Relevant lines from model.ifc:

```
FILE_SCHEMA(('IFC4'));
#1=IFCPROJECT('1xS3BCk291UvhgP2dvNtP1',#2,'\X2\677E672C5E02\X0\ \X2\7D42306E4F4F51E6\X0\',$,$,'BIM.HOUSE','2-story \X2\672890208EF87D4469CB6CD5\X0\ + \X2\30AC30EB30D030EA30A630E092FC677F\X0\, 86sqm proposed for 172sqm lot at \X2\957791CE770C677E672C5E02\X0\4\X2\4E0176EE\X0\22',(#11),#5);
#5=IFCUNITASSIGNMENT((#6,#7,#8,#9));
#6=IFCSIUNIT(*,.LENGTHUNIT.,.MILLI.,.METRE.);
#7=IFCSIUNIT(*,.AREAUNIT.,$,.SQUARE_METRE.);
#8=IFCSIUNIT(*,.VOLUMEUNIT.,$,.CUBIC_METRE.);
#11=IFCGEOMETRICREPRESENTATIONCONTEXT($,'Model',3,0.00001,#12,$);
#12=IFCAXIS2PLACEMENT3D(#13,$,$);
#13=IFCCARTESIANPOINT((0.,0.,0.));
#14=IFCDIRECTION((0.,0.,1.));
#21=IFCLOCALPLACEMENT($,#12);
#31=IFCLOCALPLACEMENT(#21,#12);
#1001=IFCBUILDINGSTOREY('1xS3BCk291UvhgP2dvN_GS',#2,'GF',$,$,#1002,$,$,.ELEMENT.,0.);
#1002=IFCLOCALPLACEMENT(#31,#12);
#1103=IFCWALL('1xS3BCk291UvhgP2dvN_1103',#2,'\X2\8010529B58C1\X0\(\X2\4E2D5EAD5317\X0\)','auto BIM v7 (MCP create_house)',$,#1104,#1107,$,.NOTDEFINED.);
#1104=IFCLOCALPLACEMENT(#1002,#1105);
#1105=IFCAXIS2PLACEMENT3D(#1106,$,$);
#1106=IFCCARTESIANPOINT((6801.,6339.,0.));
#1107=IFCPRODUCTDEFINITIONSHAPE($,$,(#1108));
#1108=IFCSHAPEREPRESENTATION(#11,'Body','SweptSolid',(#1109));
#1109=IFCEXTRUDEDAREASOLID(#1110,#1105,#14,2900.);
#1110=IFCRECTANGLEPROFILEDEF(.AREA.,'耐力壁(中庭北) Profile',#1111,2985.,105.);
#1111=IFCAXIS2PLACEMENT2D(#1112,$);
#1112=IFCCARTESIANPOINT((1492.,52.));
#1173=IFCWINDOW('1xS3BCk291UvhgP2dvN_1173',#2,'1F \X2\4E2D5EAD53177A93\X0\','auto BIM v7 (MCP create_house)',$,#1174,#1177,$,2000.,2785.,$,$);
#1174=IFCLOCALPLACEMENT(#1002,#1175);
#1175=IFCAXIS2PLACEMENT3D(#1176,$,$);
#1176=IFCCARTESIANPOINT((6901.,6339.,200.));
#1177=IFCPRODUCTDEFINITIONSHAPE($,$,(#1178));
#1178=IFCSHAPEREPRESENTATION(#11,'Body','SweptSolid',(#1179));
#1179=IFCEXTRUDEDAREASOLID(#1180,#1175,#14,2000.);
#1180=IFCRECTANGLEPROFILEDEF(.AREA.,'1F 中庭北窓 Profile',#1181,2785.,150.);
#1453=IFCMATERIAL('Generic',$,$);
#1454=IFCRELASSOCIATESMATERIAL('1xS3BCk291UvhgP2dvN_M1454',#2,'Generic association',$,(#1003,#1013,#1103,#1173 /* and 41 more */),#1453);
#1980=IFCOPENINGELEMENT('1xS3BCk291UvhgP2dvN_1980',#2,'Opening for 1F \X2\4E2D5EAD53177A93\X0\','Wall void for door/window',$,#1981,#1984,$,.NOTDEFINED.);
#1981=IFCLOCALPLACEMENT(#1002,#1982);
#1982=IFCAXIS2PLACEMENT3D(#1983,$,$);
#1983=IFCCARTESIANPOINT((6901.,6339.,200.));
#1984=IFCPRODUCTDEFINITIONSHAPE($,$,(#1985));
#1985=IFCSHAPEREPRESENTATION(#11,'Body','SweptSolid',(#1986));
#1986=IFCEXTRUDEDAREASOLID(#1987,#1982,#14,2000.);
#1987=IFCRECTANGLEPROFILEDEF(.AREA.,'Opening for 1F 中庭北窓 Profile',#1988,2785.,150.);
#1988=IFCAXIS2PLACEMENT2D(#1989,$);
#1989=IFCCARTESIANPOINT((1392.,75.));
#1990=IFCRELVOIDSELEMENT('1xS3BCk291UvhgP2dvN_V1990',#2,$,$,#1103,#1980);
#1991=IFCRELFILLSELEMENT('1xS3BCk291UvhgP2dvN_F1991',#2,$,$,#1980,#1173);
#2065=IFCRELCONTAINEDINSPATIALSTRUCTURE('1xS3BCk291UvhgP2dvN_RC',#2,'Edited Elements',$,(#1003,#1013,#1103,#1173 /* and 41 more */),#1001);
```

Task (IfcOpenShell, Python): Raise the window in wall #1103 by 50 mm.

```python
import numpy as np
import ifcopenshell
import ifcopenshell.api.geometry
import ifcopenshell.util.placement
import ifcopenshell.util.unit

model = ifcopenshell.open("model.ifc")
unit_scale = ifcopenshell.util.unit.calculate_unit_scale(model)

window = model.by_guid("1xS3BCk291UvhgP2dvN_1173")
opening = window.FillsVoids[0].RelatingOpeningElement
dz = 50.0

shift = np.array([0.0, 0.0, dz])
# The window is not placed relative to its opening, so move both.
for product in (opening, window):
    matrix = ifcopenshell.util.placement.get_local_placement(product.ObjectPlacement)
    matrix[:3, 3] += shift
    ifcopenshell.api.geometry.edit_object_placement(model, product=product, matrix=matrix, is_si=False)

print(f"moved by {dz * unit_scale:+.3f} m")

model.write("model_rev.ifc")
```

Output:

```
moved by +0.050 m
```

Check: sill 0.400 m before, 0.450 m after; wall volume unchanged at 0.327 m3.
